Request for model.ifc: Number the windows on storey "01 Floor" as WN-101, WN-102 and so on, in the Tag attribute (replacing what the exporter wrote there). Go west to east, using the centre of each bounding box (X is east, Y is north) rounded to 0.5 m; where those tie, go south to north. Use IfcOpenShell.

First a look at what the model holds.

```python
import ifcopenshell
import ifcopenshell.util.element
import ifcopenshell.util.placement

model = ifcopenshell.open("model.ifc")
print(model.schema)
storey = next(s for s in model.by_type("IfcBuildingStorey") if s.Name == "01 Floor")
windows = [e for e in ifcopenshell.util.element.get_decomposition(storey) if e.is_a("IfcWindow")]
for e in sorted(windows, key=lambda e: e.id()):
    origin = ifcopenshell.util.placement.get_local_placement(e.ObjectPlacement)[:3, 3]
    print(e.id(), e.Tag, e.Name, origin.round(2) + 0.0, sep=" | ")
```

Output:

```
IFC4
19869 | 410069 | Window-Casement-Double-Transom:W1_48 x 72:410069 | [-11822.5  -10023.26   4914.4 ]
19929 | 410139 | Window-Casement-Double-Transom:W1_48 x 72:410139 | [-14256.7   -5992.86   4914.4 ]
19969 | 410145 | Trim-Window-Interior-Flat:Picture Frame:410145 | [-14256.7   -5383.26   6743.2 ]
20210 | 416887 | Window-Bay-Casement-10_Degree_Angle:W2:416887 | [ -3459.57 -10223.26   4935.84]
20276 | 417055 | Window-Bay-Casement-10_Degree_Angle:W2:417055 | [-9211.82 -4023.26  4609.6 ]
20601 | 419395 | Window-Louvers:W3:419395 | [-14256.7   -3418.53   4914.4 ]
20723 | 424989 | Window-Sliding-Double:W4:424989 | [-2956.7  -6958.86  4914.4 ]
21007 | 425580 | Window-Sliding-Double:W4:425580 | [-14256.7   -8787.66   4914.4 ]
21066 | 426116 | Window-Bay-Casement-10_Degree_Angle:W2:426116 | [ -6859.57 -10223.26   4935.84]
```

```python
import ifcopenshell
import ifcopenshell.geom
import ifcopenshell.util.element
import ifcopenshell.util.shape

model = ifcopenshell.open("model.ifc")
settings = ifcopenshell.geom.settings()
settings.set("use-world-coords", True)


def centre(element):
    shape = ifcopenshell.geom.create_shape(settings, element)
    return ifcopenshell.util.shape.get_bbox_centroid(shape.geometry)


storey = next(s for s in model.by_type("IfcBuildingStorey") if s.Name == "01 Floor")
windows = [e for e in ifcopenshell.util.element.get_decomposition(storey) if e.is_a("IfcWindow")]

# Insertion points can sit at a corner or the storey origin, so sort by the geometry (in metres).
centres = {e: centre(e) for e in windows}
windows.sort(key=lambda e: (round(centres[e][0] / 0.5), centres[e][1]))

for i, e in enumerate(windows, start=1):
    number = f"WN-1{i:02d}"
    e.Tag = number
    print(e.id(), number)

model.write("model_rev.ifc")
```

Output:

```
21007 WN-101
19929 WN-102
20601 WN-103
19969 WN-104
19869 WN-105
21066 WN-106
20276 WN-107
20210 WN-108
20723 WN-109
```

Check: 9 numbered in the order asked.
